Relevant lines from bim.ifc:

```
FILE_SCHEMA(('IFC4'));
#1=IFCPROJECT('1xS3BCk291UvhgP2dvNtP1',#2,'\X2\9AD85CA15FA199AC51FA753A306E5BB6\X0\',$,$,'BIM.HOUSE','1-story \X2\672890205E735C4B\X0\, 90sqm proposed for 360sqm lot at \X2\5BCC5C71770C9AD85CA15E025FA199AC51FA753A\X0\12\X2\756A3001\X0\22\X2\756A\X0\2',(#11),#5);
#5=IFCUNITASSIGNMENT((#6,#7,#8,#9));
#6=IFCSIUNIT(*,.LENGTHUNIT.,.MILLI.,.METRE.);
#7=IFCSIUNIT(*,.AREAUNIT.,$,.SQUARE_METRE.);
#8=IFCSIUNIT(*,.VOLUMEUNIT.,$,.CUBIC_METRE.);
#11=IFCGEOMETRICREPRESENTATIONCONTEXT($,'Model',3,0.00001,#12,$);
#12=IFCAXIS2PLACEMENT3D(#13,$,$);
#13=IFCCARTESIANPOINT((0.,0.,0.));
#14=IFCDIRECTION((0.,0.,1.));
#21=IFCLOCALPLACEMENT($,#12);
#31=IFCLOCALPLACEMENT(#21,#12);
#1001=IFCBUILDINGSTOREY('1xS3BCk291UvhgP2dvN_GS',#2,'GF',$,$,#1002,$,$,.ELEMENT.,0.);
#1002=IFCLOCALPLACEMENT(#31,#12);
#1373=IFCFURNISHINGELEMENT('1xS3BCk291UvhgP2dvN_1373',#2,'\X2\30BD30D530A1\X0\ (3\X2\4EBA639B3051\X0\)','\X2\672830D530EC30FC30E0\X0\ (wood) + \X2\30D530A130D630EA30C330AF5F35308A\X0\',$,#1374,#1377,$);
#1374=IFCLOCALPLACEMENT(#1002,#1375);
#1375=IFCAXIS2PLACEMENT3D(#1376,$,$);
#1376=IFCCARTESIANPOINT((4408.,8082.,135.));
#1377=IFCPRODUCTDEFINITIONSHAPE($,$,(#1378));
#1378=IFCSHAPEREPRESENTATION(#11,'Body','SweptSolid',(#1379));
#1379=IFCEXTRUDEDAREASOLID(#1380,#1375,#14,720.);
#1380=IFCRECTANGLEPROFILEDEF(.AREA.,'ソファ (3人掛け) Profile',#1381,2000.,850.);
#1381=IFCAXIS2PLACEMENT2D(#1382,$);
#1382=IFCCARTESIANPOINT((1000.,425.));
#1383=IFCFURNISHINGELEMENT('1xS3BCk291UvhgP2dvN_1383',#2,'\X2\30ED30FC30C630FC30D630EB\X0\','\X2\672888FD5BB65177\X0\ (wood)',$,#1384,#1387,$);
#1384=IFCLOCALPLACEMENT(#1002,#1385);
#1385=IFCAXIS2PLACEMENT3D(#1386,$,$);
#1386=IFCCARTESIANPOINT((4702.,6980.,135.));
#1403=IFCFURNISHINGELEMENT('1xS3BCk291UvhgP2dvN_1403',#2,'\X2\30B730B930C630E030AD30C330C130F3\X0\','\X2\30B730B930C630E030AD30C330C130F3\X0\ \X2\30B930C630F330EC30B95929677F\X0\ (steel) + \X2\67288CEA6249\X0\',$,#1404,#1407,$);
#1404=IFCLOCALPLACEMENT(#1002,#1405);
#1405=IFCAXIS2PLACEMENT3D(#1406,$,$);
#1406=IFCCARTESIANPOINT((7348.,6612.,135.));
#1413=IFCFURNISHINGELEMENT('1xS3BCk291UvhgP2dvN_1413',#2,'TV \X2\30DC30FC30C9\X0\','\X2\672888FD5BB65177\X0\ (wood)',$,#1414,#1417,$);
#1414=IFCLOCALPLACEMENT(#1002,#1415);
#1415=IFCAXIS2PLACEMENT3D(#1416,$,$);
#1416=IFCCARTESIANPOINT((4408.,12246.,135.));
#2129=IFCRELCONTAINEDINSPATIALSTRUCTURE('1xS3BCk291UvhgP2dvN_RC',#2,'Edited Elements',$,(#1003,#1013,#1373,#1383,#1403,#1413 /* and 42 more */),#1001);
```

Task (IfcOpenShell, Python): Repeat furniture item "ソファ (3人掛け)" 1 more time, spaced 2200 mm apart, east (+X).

```python
import numpy as np
import ifcopenshell
import ifcopenshell.api.geometry
import ifcopenshell.api.root
import ifcopenshell.util.element
import ifcopenshell.util.placement
import ifcopenshell.util.unit

model = ifcopenshell.open("bim.ifc")
unit_scale = ifcopenshell.util.unit.calculate_unit_scale(model)


def reuse_history(source, copy):
    """copy_class also copies each property set's owner history, people and application; keep the originals."""
    for rel in copy.IsDefinedBy:
        if rel.is_a("IfcRelDefinesByProperties") and (history := rel.RelatingPropertyDefinition.OwnerHistory):
            rel.RelatingPropertyDefinition.OwnerHistory = source.OwnerHistory
            ifcopenshell.util.element.remove_deep2(model, history)


source = model.by_guid("1xS3BCk291UvhgP2dvN_1373")
base = ifcopenshell.util.placement.get_local_placement(source.ObjectPlacement)
step = np.array([1.0, 0.0, 0.0]) * 2.2 / unit_scale

for i in range(1, 2):
    copy = ifcopenshell.api.root.copy_class(model, product=source)
    copy.Representation = ifcopenshell.util.element.copy_deep(
        model, source.Representation, exclude=["IfcGeometricRepresentationContext", "IfcRepresentationMap"]
    )
    reuse_history(source, copy)
    matrix = base.copy()
    matrix[:3, 3] += i * step
    print("added at", matrix[:3, 3].round(3) + 0.0)
    ifcopenshell.api.geometry.edit_object_placement(model, product=copy, matrix=matrix, is_si=False)

model.write("bim_rev.ifc")
```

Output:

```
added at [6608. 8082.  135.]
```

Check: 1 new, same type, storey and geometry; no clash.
